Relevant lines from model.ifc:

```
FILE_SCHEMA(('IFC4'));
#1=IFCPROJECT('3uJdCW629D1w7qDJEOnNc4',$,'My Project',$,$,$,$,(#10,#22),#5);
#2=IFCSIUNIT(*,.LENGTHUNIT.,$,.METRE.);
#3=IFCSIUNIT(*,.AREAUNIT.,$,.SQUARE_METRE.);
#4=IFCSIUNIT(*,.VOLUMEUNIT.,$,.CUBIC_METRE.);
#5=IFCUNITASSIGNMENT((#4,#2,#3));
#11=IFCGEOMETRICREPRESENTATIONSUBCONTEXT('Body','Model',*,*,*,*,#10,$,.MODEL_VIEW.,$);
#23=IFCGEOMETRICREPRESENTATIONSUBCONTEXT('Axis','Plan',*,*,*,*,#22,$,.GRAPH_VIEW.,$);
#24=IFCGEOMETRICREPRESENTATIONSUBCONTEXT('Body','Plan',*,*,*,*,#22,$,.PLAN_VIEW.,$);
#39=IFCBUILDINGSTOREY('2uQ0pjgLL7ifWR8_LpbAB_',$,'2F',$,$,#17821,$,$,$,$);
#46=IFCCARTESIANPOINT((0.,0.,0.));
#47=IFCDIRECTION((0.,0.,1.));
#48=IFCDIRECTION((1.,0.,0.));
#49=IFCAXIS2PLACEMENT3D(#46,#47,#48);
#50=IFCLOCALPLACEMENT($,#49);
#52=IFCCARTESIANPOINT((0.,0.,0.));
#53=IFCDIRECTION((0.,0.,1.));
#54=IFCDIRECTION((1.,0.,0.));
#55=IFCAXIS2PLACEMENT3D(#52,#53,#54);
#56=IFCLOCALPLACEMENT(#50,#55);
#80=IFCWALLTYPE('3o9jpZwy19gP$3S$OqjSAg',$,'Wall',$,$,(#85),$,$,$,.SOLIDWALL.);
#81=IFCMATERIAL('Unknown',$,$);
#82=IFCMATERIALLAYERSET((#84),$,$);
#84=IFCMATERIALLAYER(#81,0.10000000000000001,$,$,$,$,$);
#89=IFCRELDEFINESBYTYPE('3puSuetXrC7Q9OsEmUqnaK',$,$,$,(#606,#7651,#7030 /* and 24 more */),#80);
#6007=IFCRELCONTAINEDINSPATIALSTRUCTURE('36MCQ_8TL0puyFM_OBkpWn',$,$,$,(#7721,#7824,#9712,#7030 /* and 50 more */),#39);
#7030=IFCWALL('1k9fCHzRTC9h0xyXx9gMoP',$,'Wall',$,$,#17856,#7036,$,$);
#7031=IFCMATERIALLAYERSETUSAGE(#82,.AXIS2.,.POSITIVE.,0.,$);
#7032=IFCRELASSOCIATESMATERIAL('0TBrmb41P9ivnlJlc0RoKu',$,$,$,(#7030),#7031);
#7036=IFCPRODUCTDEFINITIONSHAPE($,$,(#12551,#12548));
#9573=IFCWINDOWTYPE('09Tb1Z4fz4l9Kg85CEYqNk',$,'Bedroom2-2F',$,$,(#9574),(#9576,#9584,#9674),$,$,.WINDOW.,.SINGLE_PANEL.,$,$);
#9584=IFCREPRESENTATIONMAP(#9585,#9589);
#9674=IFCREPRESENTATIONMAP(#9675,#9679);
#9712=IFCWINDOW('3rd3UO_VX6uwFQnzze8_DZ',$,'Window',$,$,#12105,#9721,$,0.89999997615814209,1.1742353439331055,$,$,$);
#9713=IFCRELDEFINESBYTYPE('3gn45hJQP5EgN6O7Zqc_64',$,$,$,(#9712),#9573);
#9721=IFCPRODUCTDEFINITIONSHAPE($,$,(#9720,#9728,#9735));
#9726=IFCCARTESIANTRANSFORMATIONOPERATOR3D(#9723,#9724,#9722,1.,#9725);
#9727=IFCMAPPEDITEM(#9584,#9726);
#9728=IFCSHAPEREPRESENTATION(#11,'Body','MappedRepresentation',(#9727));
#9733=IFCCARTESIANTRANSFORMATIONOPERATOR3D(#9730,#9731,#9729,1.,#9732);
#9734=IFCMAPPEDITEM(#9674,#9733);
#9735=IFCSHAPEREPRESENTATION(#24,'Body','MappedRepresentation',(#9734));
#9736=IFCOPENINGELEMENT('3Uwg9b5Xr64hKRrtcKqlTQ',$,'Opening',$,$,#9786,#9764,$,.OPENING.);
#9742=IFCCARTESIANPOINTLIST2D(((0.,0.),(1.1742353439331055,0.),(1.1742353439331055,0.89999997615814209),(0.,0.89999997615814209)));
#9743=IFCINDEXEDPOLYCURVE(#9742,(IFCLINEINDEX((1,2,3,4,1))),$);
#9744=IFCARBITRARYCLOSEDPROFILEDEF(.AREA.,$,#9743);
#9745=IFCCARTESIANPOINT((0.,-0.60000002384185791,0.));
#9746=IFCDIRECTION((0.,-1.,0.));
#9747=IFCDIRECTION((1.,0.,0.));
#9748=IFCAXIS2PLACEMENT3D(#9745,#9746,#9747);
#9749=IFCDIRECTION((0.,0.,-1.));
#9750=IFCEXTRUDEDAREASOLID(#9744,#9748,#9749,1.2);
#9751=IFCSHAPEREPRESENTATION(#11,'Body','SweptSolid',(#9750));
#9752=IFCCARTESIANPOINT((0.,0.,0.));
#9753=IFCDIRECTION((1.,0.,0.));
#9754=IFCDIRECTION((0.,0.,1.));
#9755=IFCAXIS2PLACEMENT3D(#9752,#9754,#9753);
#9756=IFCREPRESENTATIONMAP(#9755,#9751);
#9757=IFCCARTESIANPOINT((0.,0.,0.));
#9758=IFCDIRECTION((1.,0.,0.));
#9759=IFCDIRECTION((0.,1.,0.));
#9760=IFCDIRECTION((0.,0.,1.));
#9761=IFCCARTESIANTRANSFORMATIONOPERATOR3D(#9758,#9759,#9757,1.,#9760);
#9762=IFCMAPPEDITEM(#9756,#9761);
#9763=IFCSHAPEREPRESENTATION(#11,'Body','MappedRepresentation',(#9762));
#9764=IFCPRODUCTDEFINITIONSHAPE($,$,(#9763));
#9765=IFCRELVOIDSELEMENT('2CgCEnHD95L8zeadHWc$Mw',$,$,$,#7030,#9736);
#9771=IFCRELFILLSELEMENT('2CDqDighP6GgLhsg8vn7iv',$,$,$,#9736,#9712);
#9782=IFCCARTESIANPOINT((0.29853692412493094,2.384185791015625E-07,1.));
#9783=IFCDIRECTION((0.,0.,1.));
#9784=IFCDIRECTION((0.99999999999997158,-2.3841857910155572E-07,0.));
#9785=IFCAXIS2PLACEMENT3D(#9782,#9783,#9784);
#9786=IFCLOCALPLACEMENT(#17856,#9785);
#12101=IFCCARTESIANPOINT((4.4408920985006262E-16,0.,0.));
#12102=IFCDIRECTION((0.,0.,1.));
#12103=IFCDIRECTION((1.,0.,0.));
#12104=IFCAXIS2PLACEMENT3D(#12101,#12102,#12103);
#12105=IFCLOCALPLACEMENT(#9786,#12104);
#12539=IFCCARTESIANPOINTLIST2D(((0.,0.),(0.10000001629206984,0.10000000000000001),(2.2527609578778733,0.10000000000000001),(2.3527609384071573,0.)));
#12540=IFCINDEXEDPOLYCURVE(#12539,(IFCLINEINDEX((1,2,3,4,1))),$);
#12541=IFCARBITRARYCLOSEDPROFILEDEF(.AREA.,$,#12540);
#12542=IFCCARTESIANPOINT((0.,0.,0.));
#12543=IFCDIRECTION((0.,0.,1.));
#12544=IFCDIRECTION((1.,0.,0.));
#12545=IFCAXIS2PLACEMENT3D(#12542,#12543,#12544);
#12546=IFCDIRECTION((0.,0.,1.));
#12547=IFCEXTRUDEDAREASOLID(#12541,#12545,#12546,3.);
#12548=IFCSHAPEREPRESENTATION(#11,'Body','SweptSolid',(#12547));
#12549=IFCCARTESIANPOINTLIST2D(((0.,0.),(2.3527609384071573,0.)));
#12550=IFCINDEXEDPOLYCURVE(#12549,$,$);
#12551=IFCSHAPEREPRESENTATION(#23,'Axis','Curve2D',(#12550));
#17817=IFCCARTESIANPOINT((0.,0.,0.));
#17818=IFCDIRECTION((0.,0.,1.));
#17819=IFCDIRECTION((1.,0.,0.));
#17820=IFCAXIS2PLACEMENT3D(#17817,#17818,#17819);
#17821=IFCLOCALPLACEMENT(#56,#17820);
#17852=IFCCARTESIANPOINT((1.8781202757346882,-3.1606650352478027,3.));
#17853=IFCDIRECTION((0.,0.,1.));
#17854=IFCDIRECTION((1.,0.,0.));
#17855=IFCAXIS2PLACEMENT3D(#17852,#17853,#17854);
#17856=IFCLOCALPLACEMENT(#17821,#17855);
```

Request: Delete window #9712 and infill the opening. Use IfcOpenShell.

```python
import ifcopenshell
import ifcopenshell.api.feature
import ifcopenshell.api.root
import ifcopenshell.geom
import ifcopenshell.util.shape

model = ifcopenshell.open("model.ifc")
settings = ifcopenshell.geom.settings()


def volume(element):
    """Net volume in cubic metres, openings subtracted."""
    shape = ifcopenshell.geom.create_shape(settings, element)
    return ifcopenshell.util.shape.get_volume(shape.geometry)


window = model.by_id(9712)
opening = window.FillsVoids[0].RelatingOpeningElement
wall = opening.VoidsElements[0].RelatingBuildingElement
before = volume(wall)

ifcopenshell.api.root.remove_product(model, product=window)
ifcopenshell.api.feature.remove_feature(model, feature=opening)

after = volume(wall)

print(f"wall volume {before:.3f} -> {after:.3f} m3")

model.write("model-out.ifc")
```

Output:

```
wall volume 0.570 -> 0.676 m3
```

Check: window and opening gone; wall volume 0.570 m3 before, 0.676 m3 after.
